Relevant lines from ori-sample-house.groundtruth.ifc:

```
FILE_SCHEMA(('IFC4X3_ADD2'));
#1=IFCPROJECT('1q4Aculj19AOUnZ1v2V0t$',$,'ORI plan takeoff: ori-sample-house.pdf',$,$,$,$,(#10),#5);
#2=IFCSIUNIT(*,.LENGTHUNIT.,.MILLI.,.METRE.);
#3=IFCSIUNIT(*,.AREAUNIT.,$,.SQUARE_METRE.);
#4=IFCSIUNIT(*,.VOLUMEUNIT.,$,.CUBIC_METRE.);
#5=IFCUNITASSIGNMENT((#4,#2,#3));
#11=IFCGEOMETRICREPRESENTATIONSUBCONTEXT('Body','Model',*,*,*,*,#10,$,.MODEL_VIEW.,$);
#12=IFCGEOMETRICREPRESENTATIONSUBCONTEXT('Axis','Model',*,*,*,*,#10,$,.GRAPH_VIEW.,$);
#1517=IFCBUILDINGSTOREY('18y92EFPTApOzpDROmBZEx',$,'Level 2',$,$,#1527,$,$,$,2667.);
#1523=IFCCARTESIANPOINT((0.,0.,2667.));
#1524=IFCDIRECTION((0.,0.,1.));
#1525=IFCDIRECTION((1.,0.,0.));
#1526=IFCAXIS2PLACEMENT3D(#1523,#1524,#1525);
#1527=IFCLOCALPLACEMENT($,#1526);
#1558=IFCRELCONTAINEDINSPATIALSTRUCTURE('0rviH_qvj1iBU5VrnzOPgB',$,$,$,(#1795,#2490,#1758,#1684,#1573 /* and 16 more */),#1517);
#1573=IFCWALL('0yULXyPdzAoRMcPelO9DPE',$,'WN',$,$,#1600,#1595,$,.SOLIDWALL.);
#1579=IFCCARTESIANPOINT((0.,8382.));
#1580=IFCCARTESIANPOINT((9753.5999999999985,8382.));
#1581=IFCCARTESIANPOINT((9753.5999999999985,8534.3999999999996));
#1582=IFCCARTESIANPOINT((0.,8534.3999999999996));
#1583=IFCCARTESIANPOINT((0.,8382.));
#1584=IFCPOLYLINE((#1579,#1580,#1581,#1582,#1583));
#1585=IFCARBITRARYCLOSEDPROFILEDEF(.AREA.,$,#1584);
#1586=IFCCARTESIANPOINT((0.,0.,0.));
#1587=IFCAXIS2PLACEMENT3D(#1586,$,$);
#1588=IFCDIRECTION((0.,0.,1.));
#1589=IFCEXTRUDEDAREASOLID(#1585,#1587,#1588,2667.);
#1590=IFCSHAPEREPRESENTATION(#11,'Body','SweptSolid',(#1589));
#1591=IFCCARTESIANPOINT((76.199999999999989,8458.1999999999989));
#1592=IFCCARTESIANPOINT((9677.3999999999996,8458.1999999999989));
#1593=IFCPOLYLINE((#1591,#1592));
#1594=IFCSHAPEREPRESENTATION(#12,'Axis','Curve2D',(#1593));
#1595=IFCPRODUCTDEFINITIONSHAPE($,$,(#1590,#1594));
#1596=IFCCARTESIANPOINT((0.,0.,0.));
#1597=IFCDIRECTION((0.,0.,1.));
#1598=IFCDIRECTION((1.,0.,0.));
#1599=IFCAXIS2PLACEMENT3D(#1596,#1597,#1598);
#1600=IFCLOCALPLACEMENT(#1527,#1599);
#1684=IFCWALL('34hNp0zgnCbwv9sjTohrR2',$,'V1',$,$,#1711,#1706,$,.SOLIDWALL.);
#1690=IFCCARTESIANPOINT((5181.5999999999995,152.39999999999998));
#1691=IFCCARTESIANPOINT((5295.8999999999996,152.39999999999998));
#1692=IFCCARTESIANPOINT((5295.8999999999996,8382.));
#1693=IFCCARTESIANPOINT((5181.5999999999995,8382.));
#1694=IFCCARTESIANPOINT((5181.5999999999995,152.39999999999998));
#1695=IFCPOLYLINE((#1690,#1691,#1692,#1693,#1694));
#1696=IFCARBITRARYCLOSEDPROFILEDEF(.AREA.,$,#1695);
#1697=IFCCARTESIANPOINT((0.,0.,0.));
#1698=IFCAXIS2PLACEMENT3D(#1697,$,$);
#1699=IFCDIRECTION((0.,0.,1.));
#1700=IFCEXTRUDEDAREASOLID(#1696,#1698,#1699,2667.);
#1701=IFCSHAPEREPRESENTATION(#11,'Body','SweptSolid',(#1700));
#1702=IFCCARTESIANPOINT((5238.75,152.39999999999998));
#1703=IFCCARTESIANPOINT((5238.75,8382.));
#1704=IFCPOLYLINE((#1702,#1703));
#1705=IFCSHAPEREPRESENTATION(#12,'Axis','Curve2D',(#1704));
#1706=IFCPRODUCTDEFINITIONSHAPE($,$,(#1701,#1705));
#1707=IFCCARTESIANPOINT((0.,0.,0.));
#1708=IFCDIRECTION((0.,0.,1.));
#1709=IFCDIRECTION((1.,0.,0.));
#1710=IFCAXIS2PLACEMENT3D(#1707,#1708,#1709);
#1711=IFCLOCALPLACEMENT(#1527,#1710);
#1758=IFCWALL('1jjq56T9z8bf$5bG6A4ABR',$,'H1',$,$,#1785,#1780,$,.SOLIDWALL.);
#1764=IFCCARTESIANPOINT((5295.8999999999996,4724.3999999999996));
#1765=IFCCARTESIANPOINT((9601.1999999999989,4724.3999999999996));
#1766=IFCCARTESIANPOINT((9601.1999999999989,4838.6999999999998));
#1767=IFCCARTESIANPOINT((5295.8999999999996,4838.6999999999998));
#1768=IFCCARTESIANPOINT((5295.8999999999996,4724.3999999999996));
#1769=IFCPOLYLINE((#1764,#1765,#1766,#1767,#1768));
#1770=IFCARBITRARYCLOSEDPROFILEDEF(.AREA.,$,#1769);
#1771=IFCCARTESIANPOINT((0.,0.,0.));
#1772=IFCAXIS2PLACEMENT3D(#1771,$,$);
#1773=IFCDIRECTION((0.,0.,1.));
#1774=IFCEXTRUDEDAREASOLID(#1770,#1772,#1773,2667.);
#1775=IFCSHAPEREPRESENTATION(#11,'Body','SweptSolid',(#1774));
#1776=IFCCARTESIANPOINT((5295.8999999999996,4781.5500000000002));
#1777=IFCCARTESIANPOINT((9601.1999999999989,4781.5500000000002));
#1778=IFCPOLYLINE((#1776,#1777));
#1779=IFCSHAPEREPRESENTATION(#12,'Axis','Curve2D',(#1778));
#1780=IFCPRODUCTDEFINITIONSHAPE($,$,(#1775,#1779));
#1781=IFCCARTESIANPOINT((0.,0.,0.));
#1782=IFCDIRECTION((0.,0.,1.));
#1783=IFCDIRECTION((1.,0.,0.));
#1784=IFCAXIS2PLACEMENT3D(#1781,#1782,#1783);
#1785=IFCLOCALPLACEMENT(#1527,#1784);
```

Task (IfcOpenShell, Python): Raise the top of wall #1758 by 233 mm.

```python
import ifcopenshell
import ifcopenshell.geom
import ifcopenshell.util.representation
import ifcopenshell.util.shape

model = ifcopenshell.open("ori-sample-house.groundtruth.ifc")
settings = ifcopenshell.geom.settings()


def volume(element):
    """Net volume in cubic metres, openings subtracted."""
    shape = ifcopenshell.geom.create_shape(settings, element)
    return ifcopenshell.util.shape.get_volume(shape.geometry)


wall = model.by_guid("1jjq56T9z8bf$5bG6A4ABR")
before = volume(wall)

body = ifcopenshell.util.representation.get_representation(wall, "Model", "Body")
solid = body.Items[0]
old_height = solid.Depth
solid.Depth += 233.0
after = volume(wall)

print(f"height {old_height:g} -> {solid.Depth:g}, volume {before:.3f} -> {after:.3f} m3")

model.write("ori-sample-house.groundtruth_v2.ifc")
```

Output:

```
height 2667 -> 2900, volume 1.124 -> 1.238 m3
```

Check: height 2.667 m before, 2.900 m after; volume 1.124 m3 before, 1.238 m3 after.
